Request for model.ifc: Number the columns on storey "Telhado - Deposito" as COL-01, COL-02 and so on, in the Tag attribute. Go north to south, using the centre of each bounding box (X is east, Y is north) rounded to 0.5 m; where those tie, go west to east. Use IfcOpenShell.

First a look at what the model holds.

```python
import ifcopenshell
import ifcopenshell.util.element
import ifcopenshell.util.placement

model = ifcopenshell.open("model.ifc")
print(model.schema)
storey = next(s for s in model.by_type("IfcBuildingStorey") if s.Name == "Telhado - Deposito")
columns = [e for e in ifcopenshell.util.element.get_decomposition(storey) if e.is_a("IfcColumn")]
for e in sorted(columns, key=lambda e: e.id()):
    origin = ifcopenshell.util.placement.get_local_placement(e.ObjectPlacement)[:3, 3]
    print(e.id(), e.Tag, e.Name, origin.round(2) + 0.0, sep=" | ")
```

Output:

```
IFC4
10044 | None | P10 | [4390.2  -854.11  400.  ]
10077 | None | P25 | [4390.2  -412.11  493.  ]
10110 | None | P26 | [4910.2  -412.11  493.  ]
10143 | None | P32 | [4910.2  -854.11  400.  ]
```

```python
import ifcopenshell
import ifcopenshell.geom
import ifcopenshell.util.element
import ifcopenshell.util.shape

model = ifcopenshell.open("model.ifc")
settings = ifcopenshell.geom.settings()
settings.set("use-world-coords", True)


def centre(element):
    shape = ifcopenshell.geom.create_shape(settings, element)
    return ifcopenshell.util.shape.get_bbox_centroid(shape.geometry)


storey = next(s for s in model.by_type("IfcBuildingStorey") if s.Name == "Telhado - Deposito")
columns = [e for e in ifcopenshell.util.element.get_decomposition(storey) if e.is_a("IfcColumn")]

# Insertion points can sit at a corner or the storey origin, so sort by the geometry (in metres).
centres = {e: centre(e) for e in columns}
columns.sort(key=lambda e: (-round(centres[e][1] / 0.5), centres[e][0]))

for i, e in enumerate(columns, start=1):
    number = f"COL-{i:02d}"
    e.Tag = number
    print(e.id(), number)

model.write("model_rev.ifc")
```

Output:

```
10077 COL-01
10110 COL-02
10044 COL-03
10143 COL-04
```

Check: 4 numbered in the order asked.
